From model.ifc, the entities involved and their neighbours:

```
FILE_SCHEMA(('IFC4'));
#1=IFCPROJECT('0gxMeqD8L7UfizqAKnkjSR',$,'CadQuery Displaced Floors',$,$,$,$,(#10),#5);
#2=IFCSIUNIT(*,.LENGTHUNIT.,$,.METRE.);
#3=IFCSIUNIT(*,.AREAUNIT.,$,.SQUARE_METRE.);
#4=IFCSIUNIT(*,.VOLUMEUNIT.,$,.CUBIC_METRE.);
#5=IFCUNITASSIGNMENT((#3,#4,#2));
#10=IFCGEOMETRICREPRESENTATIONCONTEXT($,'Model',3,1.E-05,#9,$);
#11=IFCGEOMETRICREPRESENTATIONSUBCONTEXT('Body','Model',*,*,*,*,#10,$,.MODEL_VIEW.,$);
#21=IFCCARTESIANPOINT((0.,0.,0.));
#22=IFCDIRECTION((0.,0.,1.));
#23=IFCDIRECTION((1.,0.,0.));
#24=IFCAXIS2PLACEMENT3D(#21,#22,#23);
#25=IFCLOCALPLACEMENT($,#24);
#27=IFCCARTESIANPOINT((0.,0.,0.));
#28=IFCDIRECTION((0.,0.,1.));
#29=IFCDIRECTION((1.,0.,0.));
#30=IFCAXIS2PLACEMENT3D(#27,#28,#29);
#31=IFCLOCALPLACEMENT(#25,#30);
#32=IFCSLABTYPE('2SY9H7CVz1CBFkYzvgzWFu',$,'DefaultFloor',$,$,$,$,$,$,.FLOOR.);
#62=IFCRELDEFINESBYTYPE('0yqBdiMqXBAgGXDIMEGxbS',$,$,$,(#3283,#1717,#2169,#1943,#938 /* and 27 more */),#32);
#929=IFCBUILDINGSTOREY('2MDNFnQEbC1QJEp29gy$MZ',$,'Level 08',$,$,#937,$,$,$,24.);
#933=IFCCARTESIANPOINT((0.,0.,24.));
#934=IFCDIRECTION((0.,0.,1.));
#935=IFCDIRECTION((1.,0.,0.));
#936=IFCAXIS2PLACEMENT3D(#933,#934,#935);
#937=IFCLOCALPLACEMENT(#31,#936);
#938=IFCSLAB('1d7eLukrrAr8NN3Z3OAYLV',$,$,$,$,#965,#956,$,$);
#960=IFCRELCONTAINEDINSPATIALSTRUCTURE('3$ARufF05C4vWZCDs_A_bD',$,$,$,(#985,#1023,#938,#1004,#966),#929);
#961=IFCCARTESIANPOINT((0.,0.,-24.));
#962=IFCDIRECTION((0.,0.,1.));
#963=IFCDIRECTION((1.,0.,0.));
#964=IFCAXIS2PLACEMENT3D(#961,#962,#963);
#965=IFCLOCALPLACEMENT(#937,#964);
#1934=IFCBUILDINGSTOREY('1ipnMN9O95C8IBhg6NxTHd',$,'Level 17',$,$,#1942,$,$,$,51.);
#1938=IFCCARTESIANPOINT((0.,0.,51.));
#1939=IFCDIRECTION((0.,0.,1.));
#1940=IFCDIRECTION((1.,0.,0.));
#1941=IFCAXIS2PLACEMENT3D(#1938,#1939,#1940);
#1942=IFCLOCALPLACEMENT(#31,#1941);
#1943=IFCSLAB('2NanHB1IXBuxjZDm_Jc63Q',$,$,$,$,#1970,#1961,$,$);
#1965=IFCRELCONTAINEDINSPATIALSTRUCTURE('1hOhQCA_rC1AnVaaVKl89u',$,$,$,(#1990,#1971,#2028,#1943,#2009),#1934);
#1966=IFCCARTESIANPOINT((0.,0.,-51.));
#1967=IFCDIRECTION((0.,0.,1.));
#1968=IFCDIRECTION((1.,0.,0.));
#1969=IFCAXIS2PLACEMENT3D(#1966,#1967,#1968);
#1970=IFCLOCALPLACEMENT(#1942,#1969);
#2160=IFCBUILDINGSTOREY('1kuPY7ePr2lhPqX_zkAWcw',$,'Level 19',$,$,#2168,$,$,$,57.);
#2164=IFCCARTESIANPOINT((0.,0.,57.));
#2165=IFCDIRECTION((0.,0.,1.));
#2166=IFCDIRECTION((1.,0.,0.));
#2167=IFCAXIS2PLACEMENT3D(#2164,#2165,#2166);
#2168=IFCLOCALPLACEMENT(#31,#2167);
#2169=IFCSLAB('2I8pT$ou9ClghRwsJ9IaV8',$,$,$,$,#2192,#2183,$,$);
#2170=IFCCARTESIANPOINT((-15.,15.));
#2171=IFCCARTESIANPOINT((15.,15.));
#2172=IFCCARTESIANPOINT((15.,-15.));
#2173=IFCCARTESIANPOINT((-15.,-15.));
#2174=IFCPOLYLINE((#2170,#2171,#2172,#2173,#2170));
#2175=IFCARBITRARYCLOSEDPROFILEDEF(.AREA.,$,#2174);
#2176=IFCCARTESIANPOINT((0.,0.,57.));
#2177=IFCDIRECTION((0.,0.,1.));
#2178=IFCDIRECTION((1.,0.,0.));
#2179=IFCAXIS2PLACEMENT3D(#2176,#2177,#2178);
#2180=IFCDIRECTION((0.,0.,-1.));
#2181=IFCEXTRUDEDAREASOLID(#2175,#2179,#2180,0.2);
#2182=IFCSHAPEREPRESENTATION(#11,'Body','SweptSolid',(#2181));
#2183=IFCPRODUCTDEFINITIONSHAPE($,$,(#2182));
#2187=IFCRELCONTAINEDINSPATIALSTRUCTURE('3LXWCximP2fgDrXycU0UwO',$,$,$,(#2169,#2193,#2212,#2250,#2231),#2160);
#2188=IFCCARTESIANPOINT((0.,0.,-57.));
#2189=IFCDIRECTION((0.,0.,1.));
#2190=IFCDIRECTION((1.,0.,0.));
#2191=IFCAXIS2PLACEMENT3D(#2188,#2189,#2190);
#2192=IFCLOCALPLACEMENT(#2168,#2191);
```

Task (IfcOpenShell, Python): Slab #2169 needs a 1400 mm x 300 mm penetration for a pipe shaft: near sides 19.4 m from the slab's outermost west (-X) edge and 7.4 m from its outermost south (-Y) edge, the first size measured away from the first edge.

```python
import numpy as np
import ifcopenshell
import ifcopenshell.api.feature
import ifcopenshell.api.geometry
import ifcopenshell.api.root
import ifcopenshell.geom
import ifcopenshell.util.placement
import ifcopenshell.util.representation
import ifcopenshell.util.shape
import ifcopenshell.util.unit

model = ifcopenshell.open("model.ifc")
unit_scale = ifcopenshell.util.unit.calculate_unit_scale(model)
settings = ifcopenshell.geom.settings()


def volume(element):
    """Net volume in cubic metres, openings subtracted."""
    shape = ifcopenshell.geom.create_shape(settings, element)
    return ifcopenshell.util.shape.get_volume(shape.geometry)


slab = model.by_guid("2I8pT$ou9ClghRwsJ9IaV8")
before = volume(slab)

# Extent in the slab's own axes, in metres. The edges named are its -X and -Y sides.
slab_shape = ifcopenshell.geom.create_shape(settings, slab)
vertices = ifcopenshell.util.shape.get_vertices(slab_shape.geometry)
x_min, y_min, bottom = vertices.min(axis=0)
top = vertices[:, 2].max()

opening = ifcopenshell.api.root.create_entity(model, ifc_class="IfcOpeningElement", name="Pipe shaft opening", predefined_type="OPENING")
context = ifcopenshell.util.representation.get_context(model, "Model", "Body", "MODEL_VIEW")
width, depth = 1.4, 0.3
outline = [(0.0, 0.0), (width, 0.0), (width, depth), (0.0, depth), (0.0, 0.0)]
# Overshoot both faces by 50 mm so the cut is clean.
shape = ifcopenshell.api.geometry.add_slab_representation(
    model, context=context, depth=top - bottom + 0.1, polyline=outline
)
ifcopenshell.api.geometry.assign_representation(model, product=opening, representation=shape)

matrix = ifcopenshell.util.placement.get_local_placement(slab.ObjectPlacement)
matrix[:, 3] = matrix @ np.append(np.array([x_min + 19.4, y_min + 7.4, bottom - 0.05]) / unit_scale, 1.0)
ifcopenshell.api.geometry.edit_object_placement(model, product=opening, matrix=matrix, is_si=False)
ifcopenshell.api.feature.add_feature(model, feature=opening, element=slab)

after = volume(slab)

print(f"slab volume {before:.3f} -> {after:.3f} m3")

model.write("model_v2.ifc")
```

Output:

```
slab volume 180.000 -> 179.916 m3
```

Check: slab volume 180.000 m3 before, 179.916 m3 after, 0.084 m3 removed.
